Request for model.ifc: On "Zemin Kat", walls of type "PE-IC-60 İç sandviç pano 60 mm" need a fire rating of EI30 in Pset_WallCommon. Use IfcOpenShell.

First a look at what the model holds.

```python
import ifcopenshell
import ifcopenshell.util.element

model = ifcopenshell.open("model.ifc")
print(model.schema)
storey = next(s for s in model.by_type("IfcBuildingStorey") if s.Name == "Zemin Kat")
walls = [e for e in ifcopenshell.util.element.get_decomposition(storey) if e.is_a("IfcWall")]
seen = {}
for e in walls:
    element_type = ifcopenshell.util.element.get_type(e)
    key = (element_type.Name if element_type != e and element_type else None, ifcopenshell.util.element.get_pset(e, "Pset_WallCommon", "FireRating"))
    seen[key] = seen.get(key, 0) + 1
for (name, value), count in sorted(seen.items(), key=str):
    print(count, "x", name, "|", value)
```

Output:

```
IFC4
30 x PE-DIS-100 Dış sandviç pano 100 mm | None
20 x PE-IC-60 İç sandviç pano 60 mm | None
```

```python
import ifcopenshell
import ifcopenshell.api.pset
import ifcopenshell.util.element

model = ifcopenshell.open("model.ifc")

storey = next(s for s in model.by_type("IfcBuildingStorey") if s.Name == "Zemin Kat")
walls = [e for e in ifcopenshell.util.element.get_decomposition(storey) if e.is_a("IfcWall")]

count = 0
for e in walls:
    element_type = ifcopenshell.util.element.get_type(e)
    if element_type in (None, e) or element_type.Name != "PE-IC-60 İç sandviç pano 60 mm":
        continue
    # add_pset returns the element's existing set when there is one.
    pset = ifcopenshell.api.pset.add_pset(model, product=e, name="Pset_WallCommon")
    ifcopenshell.api.pset.edit_pset(model, pset=pset, properties={"FireRating": "EI30"})
    count += 1

print(count, "walls updated")

model.write("model-out.ifc")
```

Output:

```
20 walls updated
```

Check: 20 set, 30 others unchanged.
